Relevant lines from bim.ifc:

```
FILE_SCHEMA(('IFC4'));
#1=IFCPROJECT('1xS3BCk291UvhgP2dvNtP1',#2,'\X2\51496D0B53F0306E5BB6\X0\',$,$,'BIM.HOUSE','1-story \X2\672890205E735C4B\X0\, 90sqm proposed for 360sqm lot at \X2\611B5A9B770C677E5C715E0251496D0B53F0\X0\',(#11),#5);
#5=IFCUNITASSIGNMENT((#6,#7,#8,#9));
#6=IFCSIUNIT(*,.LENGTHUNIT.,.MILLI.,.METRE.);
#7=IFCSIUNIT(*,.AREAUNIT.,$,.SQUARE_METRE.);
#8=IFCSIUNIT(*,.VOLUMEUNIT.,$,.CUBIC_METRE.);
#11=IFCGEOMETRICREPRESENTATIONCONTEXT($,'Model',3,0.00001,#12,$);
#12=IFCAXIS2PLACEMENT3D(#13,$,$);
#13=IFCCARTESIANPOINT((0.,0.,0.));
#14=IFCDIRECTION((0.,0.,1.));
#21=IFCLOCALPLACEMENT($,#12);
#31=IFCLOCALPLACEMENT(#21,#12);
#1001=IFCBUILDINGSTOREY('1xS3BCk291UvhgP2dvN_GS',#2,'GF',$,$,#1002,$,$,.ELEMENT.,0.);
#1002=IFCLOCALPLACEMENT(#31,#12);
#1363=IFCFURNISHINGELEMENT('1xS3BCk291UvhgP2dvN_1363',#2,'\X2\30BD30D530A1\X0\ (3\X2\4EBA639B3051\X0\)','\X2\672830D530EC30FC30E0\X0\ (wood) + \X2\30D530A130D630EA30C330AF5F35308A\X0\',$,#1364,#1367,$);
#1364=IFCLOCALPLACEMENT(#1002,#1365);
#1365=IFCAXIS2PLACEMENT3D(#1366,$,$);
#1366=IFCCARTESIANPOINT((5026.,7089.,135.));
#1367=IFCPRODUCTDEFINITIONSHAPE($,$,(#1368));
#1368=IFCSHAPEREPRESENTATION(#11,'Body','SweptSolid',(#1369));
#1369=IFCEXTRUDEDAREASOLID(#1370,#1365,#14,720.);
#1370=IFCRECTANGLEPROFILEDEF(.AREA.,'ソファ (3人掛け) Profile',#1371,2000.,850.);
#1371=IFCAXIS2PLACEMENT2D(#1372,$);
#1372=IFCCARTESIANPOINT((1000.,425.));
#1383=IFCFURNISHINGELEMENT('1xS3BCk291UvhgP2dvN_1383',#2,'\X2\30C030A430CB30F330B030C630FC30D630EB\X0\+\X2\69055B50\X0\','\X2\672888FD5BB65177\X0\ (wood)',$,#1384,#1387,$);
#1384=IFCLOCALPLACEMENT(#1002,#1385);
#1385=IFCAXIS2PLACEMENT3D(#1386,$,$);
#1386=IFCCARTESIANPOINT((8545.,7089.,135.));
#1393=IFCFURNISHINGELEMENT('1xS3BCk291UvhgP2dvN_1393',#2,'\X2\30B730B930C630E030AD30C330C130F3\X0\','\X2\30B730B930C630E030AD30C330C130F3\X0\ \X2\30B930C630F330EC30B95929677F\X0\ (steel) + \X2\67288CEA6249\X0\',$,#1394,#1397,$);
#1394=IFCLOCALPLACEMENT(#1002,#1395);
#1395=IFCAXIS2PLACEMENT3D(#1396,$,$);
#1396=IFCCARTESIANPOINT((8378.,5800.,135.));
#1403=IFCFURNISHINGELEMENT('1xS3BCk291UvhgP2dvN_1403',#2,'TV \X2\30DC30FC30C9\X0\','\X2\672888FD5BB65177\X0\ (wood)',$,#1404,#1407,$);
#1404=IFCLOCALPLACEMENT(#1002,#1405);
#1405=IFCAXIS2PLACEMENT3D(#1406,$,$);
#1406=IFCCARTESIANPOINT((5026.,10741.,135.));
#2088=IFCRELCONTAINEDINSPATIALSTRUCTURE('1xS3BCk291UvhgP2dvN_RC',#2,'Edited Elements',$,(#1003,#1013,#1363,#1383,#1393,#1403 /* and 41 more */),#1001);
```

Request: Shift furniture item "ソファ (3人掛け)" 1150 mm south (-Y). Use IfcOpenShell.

```python
import ifcopenshell
import ifcopenshell.api.geometry
import ifcopenshell.util.placement

model = ifcopenshell.open("bim.ifc")

item = model.by_id(1363)
matrix = ifcopenshell.util.placement.get_local_placement(item.ObjectPlacement)
matrix[1, 3] -= 1150.0
ifcopenshell.api.geometry.edit_object_placement(model, product=item, matrix=matrix, is_si=False)

print(ifcopenshell.util.placement.get_local_placement(item.ObjectPlacement).round(3) + 0.0)

model.write("bim_updated.ifc")
```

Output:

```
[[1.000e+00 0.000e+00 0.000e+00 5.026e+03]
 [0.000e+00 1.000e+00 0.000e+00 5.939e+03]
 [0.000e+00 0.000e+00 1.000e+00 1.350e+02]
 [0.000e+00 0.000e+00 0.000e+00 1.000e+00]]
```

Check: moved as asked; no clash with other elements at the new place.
